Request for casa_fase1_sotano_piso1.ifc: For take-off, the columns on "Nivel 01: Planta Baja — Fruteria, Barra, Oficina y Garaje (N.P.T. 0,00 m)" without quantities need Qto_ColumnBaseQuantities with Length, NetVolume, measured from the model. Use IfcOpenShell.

First a look at what the model holds.

```python
import ifcopenshell
import ifcopenshell.util.element
import ifcopenshell.util.unit

model = ifcopenshell.open("casa_fase1_sotano_piso1.ifc")
print(model.schema)
for unit_type in ("LENGTHUNIT", "AREAUNIT", "VOLUMEUNIT"):
    print(unit_type, ifcopenshell.util.unit.calculate_unit_scale(model, unit_type))
storey = next(s for s in model.by_type("IfcBuildingStorey") if s.Name == "Nivel 01: Planta Baja — Fruteria, Barra, Oficina y Garaje (N.P.T. 0,00 m)")
columns = [e for e in ifcopenshell.util.element.get_decomposition(storey) if e.is_a("IfcColumn")]
for e in sorted(columns, key=lambda e: e.id()):
    print(e.id(), e.is_a(), e.Name, list(ifcopenshell.util.element.get_psets(e, qtos_only=True)), sep=" | ")
```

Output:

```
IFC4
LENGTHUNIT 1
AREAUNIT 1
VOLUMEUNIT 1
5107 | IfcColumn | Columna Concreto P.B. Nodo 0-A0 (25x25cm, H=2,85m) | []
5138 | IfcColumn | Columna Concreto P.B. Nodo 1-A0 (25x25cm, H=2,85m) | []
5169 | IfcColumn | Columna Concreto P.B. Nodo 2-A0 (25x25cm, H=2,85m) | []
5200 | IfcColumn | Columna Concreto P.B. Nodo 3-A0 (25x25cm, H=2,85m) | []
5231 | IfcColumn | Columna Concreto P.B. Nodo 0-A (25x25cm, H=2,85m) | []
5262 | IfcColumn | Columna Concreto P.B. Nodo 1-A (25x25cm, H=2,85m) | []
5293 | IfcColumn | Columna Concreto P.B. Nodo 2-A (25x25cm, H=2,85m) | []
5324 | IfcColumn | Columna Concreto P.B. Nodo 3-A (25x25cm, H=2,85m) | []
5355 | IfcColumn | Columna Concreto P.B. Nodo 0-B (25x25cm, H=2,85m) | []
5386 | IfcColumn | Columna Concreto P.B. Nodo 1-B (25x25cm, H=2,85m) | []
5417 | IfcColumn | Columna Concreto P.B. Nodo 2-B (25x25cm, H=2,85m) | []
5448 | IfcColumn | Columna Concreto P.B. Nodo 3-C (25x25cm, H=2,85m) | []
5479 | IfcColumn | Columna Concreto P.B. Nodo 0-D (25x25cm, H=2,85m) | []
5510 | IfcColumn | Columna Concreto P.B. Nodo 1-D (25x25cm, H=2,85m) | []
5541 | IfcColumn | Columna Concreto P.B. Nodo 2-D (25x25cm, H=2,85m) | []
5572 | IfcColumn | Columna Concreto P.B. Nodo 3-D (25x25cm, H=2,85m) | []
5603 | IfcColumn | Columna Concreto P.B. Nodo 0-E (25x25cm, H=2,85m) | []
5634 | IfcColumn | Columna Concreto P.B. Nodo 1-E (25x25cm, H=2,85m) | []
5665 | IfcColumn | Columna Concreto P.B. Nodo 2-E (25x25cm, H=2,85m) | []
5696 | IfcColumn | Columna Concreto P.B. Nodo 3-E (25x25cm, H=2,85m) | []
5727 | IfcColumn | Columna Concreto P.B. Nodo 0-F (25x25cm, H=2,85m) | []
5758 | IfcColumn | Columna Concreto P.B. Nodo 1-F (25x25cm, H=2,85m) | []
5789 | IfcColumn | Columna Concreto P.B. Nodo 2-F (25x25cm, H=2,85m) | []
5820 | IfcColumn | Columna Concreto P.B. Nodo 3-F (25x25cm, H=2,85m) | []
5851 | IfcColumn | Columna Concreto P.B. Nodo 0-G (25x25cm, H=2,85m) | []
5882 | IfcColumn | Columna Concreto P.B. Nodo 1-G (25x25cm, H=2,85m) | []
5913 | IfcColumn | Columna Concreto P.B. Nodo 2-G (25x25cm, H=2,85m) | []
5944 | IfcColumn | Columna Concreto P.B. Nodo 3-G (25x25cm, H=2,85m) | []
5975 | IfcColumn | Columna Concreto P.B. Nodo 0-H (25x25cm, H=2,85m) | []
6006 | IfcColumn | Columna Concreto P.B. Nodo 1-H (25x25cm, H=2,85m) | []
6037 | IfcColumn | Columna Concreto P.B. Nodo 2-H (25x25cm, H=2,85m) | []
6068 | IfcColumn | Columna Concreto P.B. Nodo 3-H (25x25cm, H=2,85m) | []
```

```python
import ifcopenshell
import ifcopenshell.api.pset
import ifcopenshell.geom
import ifcopenshell.util.element
import ifcopenshell.util.shape
import ifcopenshell.util.unit

model = ifcopenshell.open("casa_fase1_sotano_piso1.ifc")
unit_scale = ifcopenshell.util.unit.calculate_unit_scale(model)
volume_scale = ifcopenshell.util.unit.calculate_unit_scale(model, "VOLUMEUNIT")
settings = ifcopenshell.geom.settings()

storey = next(s for s in model.by_type("IfcBuildingStorey") if s.Name == "Nivel 01: Planta Baja — Fruteria, Barra, Oficina y Garaje (N.P.T. 0,00 m)")
columns = [e for e in ifcopenshell.util.element.get_decomposition(storey) if e.is_a("IfcColumn")]

for e in sorted(columns, key=lambda e: e.id()):
    if ifcopenshell.util.element.get_psets(e, qtos_only=True, should_inherit=False):
        continue
    # Geometry comes back in metres, in the element's own axes.
    shape = ifcopenshell.geom.create_shape(settings, e)
    values = {
        "Length": ifcopenshell.util.shape.get_z(shape.geometry) / unit_scale,
        "NetVolume": ifcopenshell.util.shape.get_volume(shape.geometry) / volume_scale,
    }
    qto = ifcopenshell.api.pset.add_qto(model, product=e, name="Qto_ColumnBaseQuantities")
    ifcopenshell.api.pset.edit_qto(model, qto=qto, properties=values)
    print(e.id(), {k: round(v, 3) for k, v in values.items()})

model.write("casa_fase1_sotano_piso1_rev.ifc")
```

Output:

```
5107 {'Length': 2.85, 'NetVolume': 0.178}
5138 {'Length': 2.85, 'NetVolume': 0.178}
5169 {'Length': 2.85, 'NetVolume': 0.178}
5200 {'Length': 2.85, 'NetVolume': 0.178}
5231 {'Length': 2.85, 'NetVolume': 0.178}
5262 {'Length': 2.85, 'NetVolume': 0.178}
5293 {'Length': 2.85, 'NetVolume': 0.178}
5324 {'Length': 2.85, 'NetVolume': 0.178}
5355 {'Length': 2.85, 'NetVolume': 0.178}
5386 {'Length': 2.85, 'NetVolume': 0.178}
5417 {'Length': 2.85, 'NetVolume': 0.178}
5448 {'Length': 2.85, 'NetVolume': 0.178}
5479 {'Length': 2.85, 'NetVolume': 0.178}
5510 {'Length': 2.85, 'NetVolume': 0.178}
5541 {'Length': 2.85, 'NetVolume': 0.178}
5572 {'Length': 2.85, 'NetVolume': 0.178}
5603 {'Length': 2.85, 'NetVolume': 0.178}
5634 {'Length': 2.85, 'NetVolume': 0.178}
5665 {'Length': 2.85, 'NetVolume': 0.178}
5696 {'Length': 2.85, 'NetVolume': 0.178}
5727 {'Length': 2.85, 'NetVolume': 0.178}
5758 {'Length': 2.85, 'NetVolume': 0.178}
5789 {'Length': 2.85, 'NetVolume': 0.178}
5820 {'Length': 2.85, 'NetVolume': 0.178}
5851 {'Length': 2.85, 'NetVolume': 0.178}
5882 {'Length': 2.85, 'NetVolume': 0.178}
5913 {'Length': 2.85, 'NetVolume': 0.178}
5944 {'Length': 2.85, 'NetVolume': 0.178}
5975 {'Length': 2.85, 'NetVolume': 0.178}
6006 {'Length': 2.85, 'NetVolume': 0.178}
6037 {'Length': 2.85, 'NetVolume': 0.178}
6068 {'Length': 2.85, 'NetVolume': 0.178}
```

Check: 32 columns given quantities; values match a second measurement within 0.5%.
